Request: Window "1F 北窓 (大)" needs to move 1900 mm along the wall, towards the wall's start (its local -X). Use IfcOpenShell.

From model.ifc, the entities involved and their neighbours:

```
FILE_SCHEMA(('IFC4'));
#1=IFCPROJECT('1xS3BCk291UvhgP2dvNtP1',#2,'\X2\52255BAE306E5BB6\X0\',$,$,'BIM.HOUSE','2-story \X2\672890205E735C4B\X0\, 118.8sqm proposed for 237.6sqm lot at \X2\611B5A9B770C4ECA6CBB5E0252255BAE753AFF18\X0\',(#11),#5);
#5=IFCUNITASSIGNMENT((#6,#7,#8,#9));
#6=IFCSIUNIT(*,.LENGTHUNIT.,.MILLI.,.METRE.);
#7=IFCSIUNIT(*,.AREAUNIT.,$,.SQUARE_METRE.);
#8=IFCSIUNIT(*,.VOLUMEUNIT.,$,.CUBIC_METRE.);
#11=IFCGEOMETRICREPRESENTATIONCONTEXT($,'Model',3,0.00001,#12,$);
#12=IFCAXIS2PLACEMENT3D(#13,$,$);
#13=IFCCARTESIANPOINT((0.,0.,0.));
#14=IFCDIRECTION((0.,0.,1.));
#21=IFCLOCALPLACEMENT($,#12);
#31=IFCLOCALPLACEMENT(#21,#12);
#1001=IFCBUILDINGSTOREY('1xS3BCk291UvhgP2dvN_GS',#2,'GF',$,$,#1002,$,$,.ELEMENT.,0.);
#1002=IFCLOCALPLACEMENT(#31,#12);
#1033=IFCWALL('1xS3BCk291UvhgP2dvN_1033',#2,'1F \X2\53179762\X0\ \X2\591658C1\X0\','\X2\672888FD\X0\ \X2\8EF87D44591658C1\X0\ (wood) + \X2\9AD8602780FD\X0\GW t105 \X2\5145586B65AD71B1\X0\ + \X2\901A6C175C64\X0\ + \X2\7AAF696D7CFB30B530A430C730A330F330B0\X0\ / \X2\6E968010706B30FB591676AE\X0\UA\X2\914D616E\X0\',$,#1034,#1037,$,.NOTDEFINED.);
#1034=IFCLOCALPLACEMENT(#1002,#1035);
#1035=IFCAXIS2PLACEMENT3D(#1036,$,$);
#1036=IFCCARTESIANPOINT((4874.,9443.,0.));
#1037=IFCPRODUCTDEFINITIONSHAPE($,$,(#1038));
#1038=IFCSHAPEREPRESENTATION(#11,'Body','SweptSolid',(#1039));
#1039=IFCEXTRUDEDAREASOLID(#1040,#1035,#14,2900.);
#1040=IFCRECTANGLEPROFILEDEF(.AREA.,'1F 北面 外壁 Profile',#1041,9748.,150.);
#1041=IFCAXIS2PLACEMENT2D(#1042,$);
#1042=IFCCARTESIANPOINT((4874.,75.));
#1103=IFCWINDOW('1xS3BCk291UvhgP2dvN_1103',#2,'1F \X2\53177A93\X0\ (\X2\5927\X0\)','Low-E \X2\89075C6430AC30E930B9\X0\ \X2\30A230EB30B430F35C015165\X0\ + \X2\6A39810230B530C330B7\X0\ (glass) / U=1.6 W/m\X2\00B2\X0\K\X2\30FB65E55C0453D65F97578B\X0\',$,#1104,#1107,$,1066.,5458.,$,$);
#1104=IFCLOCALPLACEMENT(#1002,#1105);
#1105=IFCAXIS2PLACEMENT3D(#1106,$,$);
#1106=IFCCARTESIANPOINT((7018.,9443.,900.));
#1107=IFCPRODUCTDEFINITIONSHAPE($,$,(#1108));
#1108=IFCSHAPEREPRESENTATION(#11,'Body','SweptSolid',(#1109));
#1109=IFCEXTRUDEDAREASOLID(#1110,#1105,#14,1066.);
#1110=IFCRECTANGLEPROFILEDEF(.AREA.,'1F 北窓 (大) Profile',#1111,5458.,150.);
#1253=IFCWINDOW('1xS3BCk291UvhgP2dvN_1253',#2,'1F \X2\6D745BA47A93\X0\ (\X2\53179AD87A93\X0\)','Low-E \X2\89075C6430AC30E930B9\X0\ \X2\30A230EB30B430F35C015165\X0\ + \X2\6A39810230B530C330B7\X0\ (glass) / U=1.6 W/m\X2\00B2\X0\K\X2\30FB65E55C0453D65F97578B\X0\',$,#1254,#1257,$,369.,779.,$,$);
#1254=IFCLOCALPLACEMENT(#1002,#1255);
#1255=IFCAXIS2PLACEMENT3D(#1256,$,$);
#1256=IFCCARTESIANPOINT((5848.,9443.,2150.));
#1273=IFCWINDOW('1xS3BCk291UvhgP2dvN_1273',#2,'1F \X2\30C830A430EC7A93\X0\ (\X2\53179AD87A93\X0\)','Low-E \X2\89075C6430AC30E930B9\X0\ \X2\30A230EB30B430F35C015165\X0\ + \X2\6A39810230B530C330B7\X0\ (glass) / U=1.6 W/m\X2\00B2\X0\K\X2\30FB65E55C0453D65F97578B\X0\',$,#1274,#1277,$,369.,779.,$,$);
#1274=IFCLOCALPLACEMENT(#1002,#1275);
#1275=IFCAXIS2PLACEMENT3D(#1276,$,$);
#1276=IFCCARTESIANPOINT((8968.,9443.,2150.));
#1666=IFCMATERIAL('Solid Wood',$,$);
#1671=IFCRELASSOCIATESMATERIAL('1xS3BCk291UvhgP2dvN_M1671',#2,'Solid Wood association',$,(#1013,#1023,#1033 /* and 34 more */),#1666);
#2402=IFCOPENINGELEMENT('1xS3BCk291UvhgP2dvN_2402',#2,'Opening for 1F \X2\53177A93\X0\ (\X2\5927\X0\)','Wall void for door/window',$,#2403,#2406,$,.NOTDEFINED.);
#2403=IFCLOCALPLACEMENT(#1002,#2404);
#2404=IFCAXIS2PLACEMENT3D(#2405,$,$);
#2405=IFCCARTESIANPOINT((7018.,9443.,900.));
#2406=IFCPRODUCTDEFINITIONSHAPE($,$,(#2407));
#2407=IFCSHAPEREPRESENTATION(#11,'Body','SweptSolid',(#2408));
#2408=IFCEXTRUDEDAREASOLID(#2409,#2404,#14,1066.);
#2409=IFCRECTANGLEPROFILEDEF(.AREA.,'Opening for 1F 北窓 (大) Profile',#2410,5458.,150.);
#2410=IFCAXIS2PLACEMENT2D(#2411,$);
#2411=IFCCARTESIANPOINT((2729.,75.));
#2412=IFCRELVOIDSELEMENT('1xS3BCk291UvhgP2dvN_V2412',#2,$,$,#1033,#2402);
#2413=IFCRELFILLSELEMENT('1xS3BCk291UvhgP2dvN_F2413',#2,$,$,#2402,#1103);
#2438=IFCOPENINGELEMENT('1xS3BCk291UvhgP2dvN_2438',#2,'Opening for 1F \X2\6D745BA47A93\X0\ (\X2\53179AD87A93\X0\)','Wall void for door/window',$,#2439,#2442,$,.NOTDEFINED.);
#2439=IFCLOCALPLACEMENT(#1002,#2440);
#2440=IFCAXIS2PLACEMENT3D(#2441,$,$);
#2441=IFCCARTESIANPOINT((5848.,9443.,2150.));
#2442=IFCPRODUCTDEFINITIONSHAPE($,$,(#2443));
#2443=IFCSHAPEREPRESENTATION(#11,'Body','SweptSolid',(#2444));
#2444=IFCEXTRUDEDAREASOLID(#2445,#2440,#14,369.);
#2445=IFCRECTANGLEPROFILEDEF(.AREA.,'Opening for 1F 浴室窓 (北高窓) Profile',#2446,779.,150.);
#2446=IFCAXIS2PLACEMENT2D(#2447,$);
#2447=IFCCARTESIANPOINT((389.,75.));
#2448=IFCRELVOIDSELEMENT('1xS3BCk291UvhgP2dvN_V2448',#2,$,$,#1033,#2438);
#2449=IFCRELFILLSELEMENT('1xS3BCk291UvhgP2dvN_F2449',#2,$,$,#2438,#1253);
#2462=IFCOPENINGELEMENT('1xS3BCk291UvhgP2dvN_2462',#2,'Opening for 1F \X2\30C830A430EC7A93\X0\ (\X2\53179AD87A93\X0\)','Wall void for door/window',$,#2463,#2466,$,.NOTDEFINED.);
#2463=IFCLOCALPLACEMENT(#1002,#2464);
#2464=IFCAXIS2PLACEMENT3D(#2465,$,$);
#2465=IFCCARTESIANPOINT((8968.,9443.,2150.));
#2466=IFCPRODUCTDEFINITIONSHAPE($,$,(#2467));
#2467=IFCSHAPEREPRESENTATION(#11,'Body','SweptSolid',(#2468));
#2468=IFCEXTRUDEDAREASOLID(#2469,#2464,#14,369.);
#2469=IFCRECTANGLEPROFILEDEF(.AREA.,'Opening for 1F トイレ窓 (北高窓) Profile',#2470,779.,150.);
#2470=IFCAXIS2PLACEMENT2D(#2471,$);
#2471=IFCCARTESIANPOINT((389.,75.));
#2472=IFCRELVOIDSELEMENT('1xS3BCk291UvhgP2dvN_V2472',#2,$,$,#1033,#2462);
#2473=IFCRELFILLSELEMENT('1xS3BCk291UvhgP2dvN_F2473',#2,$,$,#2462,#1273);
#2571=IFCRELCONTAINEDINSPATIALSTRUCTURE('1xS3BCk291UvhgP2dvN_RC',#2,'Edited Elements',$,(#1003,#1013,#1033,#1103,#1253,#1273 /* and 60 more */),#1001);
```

```python
import ifcopenshell
import ifcopenshell.api.geometry
import ifcopenshell.util.placement
import ifcopenshell.util.unit

model = ifcopenshell.open("model.ifc")
unit_scale = ifcopenshell.util.unit.calculate_unit_scale(model)

window = model.by_guid("1xS3BCk291UvhgP2dvN_1103")
opening = window.FillsVoids[0].RelatingOpeningElement
wall = opening.VoidsElements[0].RelatingBuildingElement

wall_matrix = ifcopenshell.util.placement.get_local_placement(wall.ObjectPlacement)
shift = wall_matrix[:3, 0] * -1.9 / unit_scale
before = ifcopenshell.util.placement.get_local_placement(window.ObjectPlacement)[:3, 3].copy()

# The window is not placed relative to its opening, so move both.
for product in (opening, window):
    matrix = ifcopenshell.util.placement.get_local_placement(product.ObjectPlacement)
    matrix[:3, 3] += shift
    ifcopenshell.api.geometry.edit_object_placement(model, product=product, matrix=matrix, is_si=False)

after = ifcopenshell.util.placement.get_local_placement(window.ObjectPlacement)[:3, 3]
print("window moved by", (after - before).round(3) + 0.0)

model.write("model_updated.ifc")
```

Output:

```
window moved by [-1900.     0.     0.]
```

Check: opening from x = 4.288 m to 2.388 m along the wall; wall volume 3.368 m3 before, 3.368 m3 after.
